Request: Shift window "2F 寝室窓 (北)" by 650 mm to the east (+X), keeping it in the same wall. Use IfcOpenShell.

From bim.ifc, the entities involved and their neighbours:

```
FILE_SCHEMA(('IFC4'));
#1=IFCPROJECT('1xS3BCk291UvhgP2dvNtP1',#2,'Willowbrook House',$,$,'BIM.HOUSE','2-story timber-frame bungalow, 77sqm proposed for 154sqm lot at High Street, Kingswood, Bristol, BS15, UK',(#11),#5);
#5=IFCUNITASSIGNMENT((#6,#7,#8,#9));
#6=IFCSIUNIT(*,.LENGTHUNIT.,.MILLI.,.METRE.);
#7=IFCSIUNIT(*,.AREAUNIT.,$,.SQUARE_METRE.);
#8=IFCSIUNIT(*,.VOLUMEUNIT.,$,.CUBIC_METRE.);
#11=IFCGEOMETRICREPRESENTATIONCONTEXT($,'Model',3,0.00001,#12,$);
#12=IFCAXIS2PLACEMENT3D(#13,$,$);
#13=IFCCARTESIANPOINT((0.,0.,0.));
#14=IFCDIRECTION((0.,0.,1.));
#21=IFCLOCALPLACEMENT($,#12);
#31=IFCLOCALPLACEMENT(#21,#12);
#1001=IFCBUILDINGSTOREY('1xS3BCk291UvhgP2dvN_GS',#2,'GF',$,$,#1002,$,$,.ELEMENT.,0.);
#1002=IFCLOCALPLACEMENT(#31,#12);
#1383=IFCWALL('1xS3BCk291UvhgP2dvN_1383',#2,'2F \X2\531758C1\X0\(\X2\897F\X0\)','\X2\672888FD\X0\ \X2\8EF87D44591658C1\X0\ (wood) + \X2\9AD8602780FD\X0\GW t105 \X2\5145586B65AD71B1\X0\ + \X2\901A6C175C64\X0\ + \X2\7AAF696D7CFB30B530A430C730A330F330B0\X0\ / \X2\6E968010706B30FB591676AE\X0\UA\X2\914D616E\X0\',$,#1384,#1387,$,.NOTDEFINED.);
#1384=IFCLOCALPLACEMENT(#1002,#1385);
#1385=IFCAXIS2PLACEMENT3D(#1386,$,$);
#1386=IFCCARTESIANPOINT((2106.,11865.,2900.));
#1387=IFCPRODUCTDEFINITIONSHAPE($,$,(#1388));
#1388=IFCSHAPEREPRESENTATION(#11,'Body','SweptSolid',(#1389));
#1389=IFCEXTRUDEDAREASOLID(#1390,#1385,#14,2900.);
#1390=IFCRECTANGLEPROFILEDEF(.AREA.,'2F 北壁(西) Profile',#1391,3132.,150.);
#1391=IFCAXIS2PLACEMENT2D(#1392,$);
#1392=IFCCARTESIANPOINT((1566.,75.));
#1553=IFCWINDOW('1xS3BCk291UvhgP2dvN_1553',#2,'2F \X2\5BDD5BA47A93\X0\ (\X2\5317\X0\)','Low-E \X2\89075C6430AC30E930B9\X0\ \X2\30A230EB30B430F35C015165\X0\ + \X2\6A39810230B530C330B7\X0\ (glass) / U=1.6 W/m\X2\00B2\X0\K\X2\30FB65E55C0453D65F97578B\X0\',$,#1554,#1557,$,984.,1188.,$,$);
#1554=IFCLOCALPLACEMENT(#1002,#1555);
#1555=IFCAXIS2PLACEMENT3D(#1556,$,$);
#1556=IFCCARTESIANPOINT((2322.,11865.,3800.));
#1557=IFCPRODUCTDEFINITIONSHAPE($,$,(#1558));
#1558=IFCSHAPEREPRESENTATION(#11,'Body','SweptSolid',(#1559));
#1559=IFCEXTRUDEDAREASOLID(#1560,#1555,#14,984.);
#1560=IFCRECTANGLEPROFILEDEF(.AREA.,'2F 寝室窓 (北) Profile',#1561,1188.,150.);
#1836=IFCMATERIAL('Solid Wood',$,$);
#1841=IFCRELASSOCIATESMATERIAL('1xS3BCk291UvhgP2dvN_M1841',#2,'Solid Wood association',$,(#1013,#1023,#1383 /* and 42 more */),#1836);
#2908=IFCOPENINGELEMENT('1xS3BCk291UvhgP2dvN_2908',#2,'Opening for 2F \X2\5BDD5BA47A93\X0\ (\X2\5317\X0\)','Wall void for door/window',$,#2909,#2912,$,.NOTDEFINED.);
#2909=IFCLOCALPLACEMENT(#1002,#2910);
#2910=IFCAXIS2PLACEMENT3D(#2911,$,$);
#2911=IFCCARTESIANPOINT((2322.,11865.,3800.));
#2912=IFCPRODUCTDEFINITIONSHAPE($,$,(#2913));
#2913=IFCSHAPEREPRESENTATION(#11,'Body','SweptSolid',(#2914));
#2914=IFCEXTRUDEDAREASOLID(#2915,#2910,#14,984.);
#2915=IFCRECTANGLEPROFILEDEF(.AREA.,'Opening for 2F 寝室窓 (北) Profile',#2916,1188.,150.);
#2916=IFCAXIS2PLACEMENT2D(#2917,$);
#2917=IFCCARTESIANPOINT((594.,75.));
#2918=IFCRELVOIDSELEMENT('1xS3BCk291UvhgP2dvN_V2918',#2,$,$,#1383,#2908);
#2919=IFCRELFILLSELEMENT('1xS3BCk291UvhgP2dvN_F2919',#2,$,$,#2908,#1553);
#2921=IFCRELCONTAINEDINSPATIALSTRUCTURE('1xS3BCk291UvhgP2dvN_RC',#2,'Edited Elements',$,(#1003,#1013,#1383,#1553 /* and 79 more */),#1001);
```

```python
import ifcopenshell
import ifcopenshell.api.geometry
import ifcopenshell.util.placement

model = ifcopenshell.open("bim.ifc")

window = model.by_guid("1xS3BCk291UvhgP2dvN_1553")
opening = window.FillsVoids[0].RelatingOpeningElement
wall = opening.VoidsElements[0].RelatingBuildingElement

wall_matrix = ifcopenshell.util.placement.get_local_placement(wall.ObjectPlacement)
shift = wall_matrix[:3, 0] * 650.0
before = ifcopenshell.util.placement.get_local_placement(window.ObjectPlacement)[:3, 3].copy()

# The window is not placed relative to its opening, so move both.
for product in (opening, window):
    matrix = ifcopenshell.util.placement.get_local_placement(product.ObjectPlacement)
    matrix[:3, 3] += shift
    ifcopenshell.api.geometry.edit_object_placement(model, product=product, matrix=matrix, is_si=False)

after = ifcopenshell.util.placement.get_local_placement(window.ObjectPlacement)[:3, 3]
print("window moved by", (after - before).round(3) + 0.0)

model.write("bim_updated.ifc")
```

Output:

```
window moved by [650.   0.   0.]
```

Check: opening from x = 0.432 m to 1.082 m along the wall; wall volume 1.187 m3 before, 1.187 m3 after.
